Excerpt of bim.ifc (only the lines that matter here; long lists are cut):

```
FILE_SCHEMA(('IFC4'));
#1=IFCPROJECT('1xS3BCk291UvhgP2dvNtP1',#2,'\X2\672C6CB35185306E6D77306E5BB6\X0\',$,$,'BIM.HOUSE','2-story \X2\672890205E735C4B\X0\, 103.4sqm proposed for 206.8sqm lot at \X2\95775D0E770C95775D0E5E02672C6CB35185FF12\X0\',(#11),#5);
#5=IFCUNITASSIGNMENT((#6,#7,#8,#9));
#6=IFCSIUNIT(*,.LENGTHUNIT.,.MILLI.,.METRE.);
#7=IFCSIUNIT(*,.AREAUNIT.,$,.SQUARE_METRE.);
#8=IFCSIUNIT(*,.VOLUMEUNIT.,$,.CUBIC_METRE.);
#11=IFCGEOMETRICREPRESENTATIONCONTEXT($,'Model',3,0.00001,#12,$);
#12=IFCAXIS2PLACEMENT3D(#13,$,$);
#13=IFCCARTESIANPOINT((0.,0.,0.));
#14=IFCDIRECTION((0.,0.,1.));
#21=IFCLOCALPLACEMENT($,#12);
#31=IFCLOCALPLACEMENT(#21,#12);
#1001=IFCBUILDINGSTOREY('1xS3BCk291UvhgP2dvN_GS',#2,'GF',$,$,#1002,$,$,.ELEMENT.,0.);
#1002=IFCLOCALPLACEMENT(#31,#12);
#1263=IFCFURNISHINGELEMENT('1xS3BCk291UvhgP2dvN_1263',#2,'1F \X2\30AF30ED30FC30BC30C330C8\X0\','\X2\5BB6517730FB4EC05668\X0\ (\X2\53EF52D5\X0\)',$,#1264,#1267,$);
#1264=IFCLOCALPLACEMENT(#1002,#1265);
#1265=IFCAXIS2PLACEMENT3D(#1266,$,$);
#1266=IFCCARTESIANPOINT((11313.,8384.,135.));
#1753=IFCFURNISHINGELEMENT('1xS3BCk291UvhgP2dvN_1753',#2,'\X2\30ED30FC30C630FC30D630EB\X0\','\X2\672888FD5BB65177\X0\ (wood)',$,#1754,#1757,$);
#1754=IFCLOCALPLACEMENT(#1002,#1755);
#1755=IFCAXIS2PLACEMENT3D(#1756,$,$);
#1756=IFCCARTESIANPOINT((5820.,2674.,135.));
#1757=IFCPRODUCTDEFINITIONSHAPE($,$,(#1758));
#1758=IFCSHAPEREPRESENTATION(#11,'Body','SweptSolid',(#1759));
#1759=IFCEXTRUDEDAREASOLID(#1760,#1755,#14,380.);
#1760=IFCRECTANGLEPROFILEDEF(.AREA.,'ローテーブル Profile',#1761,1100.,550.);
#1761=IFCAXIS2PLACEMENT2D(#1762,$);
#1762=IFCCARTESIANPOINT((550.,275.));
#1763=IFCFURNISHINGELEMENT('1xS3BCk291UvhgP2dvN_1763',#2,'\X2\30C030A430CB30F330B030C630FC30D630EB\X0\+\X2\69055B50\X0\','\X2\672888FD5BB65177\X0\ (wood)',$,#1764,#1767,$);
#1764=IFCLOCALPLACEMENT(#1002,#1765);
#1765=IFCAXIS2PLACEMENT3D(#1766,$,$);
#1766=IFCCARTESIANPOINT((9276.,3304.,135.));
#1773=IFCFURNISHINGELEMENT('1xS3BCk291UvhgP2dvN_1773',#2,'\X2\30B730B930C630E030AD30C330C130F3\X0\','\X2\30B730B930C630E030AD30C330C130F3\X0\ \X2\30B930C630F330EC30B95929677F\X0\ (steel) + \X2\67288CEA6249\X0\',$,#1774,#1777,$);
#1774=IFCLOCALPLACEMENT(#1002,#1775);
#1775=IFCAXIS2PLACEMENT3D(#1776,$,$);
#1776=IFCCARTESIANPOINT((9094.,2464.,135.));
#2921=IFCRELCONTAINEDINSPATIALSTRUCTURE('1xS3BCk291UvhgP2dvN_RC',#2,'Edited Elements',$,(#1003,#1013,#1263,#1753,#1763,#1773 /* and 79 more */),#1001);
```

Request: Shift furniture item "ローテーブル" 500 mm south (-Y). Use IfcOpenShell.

```python
import ifcopenshell
import ifcopenshell.api.geometry
import ifcopenshell.util.placement
import ifcopenshell.util.unit

model = ifcopenshell.open("bim.ifc")
unit_scale = ifcopenshell.util.unit.calculate_unit_scale(model)

item = model.by_id(1753)
matrix = ifcopenshell.util.placement.get_local_placement(item.ObjectPlacement)
matrix[1, 3] -= 0.5 / unit_scale
ifcopenshell.api.geometry.edit_object_placement(model, product=item, matrix=matrix, is_si=False)

print(ifcopenshell.util.placement.get_local_placement(item.ObjectPlacement).round(3) + 0.0)

model.write("bim-out.ifc")
```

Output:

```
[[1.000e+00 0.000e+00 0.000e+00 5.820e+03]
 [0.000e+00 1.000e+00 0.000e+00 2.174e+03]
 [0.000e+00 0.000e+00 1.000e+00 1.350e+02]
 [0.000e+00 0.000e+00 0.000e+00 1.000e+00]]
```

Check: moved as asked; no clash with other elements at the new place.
